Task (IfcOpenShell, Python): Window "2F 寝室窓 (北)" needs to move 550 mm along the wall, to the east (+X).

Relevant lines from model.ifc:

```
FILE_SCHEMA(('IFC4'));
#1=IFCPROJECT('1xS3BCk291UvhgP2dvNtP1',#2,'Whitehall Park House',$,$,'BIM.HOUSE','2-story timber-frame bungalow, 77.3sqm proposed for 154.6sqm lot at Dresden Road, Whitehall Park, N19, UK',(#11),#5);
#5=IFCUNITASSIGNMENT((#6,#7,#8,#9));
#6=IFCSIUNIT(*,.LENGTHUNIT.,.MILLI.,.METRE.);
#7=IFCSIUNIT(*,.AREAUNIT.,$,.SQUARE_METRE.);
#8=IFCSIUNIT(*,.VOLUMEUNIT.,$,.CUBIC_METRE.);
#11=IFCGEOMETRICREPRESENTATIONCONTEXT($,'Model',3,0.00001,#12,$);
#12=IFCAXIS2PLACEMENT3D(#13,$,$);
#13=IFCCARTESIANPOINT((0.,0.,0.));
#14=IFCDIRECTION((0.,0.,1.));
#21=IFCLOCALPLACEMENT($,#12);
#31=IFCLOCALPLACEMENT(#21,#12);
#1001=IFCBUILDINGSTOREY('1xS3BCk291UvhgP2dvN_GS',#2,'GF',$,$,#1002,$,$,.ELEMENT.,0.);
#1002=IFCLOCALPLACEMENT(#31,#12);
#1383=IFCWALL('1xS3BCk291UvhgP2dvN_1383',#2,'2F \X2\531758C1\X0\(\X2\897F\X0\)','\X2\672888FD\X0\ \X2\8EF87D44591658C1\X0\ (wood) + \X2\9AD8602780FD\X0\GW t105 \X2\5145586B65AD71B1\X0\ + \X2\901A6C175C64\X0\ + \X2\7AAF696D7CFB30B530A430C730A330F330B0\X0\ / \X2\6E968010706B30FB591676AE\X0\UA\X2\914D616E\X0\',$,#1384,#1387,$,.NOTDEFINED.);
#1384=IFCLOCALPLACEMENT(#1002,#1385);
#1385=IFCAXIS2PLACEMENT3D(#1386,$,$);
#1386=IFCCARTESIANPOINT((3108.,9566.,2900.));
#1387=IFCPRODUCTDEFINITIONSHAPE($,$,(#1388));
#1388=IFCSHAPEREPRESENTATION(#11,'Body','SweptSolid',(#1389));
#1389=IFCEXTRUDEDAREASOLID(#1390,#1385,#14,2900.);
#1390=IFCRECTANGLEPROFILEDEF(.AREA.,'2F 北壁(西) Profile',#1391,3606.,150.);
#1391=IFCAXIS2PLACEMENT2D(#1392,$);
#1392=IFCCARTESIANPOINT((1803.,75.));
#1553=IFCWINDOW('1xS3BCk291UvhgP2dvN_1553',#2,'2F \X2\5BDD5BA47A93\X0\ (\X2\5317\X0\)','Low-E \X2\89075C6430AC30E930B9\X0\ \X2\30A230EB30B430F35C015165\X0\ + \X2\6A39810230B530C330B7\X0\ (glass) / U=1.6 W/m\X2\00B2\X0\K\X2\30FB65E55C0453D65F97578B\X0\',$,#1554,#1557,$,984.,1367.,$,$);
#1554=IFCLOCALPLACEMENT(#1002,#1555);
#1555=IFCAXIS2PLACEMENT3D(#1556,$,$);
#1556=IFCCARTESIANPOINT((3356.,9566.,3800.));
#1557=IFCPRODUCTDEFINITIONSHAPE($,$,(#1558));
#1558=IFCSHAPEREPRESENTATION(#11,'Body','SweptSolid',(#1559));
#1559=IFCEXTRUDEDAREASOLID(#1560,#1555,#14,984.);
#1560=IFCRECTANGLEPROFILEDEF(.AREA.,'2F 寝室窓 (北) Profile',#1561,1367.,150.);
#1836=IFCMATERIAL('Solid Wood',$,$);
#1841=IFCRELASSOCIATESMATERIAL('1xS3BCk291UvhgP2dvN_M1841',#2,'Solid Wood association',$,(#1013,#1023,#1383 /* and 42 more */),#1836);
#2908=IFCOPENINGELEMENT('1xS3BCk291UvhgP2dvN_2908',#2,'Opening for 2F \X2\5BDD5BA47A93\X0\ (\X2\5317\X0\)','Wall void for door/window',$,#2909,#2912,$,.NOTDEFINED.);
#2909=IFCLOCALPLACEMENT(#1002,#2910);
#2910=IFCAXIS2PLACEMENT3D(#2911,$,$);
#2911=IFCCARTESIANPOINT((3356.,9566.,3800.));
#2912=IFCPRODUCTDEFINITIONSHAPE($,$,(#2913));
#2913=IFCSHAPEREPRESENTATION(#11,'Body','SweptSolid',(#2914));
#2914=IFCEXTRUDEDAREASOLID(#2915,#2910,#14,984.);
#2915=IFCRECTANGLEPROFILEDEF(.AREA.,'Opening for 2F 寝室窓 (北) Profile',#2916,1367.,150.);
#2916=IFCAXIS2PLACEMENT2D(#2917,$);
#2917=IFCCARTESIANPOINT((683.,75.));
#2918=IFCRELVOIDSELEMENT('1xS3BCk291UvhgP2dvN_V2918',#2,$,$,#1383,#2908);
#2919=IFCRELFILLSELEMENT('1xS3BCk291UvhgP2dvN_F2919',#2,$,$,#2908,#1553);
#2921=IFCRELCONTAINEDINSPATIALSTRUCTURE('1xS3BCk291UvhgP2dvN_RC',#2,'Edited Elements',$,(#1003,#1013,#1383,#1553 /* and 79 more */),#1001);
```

```python
import ifcopenshell
import ifcopenshell.api.geometry
import ifcopenshell.util.placement
import ifcopenshell.util.unit

model = ifcopenshell.open("model.ifc")
unit_scale = ifcopenshell.util.unit.calculate_unit_scale(model)

window = model.by_id(1553)
opening = window.FillsVoids[0].RelatingOpeningElement
wall = opening.VoidsElements[0].RelatingBuildingElement

wall_matrix = ifcopenshell.util.placement.get_local_placement(wall.ObjectPlacement)
shift = wall_matrix[:3, 0] * 0.55 / unit_scale
before = ifcopenshell.util.placement.get_local_placement(window.ObjectPlacement)[:3, 3].copy()

# The window is not placed relative to its opening, so move both.
for product in (opening, window):
    matrix = ifcopenshell.util.placement.get_local_placement(product.ObjectPlacement)
    matrix[:3, 3] += shift
    ifcopenshell.api.geometry.edit_object_placement(model, product=product, matrix=matrix, is_si=False)

after = ifcopenshell.util.placement.get_local_placement(window.ObjectPlacement)[:3, 3]
print("window moved by", (after - before).round(3) + 0.0)

model.write("model_rev.ifc")
```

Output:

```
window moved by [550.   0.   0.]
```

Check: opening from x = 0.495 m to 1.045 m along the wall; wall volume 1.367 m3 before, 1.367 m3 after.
